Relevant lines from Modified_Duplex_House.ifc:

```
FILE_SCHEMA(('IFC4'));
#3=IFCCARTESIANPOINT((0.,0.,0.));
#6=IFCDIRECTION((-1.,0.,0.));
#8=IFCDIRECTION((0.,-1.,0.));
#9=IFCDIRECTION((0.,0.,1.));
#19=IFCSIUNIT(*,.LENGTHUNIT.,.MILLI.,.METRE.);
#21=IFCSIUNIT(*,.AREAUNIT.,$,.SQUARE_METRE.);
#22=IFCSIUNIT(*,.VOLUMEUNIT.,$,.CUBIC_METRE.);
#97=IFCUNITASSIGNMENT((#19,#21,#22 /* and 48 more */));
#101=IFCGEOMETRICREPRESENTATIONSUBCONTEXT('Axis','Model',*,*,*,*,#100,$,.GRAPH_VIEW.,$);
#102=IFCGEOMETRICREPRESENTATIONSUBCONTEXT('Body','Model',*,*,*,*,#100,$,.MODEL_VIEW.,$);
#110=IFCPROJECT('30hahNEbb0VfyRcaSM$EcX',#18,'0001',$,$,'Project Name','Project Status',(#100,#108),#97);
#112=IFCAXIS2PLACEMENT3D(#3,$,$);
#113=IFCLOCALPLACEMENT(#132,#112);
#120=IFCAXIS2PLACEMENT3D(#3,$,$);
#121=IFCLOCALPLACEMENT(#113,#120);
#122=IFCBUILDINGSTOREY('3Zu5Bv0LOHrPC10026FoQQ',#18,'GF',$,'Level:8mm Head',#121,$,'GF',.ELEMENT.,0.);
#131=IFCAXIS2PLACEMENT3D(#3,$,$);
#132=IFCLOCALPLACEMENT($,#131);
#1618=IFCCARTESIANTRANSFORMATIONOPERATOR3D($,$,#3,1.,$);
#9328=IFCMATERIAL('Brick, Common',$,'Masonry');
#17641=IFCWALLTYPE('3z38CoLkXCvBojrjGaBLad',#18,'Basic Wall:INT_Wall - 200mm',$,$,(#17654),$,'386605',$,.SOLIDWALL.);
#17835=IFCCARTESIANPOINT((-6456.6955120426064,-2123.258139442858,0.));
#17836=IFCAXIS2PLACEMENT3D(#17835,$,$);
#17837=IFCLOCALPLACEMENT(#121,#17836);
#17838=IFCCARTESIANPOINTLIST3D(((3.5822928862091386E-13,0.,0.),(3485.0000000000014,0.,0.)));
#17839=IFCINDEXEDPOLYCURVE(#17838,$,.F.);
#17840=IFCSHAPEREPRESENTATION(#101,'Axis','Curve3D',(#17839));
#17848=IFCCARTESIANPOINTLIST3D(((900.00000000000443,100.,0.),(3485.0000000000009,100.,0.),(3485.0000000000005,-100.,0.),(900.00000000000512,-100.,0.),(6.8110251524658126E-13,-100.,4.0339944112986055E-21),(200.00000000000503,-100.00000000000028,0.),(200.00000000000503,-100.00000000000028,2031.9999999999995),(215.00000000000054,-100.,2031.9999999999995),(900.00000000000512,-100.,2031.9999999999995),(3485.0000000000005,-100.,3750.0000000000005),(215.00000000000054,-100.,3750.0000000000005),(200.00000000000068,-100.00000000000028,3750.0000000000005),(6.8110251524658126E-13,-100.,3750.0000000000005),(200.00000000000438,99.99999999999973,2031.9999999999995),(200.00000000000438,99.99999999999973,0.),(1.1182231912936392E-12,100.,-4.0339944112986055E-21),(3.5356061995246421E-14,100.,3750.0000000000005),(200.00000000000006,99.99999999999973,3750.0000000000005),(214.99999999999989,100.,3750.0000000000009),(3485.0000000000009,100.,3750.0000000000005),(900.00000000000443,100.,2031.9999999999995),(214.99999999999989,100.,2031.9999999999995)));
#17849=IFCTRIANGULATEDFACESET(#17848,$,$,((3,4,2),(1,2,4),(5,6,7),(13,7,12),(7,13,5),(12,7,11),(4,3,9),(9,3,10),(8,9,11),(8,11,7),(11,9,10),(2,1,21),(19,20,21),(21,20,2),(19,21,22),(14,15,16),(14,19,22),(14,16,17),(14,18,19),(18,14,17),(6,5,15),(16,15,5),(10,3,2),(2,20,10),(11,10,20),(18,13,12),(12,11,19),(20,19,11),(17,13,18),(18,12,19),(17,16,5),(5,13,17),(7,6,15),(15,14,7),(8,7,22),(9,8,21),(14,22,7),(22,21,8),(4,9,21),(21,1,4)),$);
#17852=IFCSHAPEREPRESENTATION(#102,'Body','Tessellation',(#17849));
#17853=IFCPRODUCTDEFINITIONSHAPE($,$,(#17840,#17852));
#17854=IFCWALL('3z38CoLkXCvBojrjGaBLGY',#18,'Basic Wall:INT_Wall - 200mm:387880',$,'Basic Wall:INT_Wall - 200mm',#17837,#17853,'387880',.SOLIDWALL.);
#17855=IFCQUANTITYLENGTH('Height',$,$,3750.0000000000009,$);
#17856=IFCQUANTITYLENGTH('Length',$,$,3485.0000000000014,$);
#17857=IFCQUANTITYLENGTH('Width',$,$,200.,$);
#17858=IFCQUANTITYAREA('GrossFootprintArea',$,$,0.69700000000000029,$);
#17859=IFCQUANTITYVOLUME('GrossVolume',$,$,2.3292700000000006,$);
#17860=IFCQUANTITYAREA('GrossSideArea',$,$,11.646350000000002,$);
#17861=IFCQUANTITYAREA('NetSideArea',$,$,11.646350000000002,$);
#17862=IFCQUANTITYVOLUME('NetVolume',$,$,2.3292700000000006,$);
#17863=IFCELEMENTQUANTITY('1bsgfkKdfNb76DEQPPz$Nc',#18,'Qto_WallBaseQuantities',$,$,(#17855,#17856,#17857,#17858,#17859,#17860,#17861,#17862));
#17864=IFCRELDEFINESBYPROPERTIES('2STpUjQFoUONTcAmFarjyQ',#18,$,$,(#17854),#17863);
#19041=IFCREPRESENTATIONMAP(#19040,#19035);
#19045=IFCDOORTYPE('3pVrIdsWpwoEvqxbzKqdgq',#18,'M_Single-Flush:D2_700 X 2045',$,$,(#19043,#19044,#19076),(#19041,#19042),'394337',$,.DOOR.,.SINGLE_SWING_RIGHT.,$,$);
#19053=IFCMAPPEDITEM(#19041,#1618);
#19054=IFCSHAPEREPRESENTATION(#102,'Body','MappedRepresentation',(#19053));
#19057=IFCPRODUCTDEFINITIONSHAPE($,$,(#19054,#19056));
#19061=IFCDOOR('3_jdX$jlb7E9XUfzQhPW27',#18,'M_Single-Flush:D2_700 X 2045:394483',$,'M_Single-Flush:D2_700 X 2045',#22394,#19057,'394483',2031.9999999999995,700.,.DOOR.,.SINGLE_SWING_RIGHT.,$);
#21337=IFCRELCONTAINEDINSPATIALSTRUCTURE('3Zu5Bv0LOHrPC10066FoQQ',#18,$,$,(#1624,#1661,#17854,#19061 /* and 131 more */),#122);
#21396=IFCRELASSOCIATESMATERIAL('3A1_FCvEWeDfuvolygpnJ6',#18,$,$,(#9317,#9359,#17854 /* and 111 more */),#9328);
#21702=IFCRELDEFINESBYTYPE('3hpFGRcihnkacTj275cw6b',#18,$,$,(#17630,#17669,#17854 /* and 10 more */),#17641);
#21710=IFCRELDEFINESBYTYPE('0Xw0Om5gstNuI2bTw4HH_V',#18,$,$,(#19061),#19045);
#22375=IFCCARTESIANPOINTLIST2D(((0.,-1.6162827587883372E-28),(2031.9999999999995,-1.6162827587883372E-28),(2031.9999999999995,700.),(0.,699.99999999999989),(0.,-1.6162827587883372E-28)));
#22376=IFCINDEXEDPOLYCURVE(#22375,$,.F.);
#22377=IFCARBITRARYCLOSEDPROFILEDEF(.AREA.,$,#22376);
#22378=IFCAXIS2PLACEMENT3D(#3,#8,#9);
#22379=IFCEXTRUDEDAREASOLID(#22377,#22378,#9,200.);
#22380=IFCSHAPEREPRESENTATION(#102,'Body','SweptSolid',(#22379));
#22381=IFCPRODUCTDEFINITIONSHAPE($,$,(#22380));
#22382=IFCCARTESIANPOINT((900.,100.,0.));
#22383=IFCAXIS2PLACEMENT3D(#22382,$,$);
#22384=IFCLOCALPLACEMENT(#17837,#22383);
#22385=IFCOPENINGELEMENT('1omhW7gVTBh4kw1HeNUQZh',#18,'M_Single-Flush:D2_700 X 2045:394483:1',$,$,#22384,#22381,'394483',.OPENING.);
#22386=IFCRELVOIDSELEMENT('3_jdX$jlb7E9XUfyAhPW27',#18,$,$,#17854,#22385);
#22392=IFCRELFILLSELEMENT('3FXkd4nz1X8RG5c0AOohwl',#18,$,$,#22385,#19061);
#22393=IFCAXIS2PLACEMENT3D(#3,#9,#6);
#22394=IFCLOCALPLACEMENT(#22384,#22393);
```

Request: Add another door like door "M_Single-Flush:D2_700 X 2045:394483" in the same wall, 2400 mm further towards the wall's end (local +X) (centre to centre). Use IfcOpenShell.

```python
import ifcopenshell
import ifcopenshell.api.feature
import ifcopenshell.api.geometry
import ifcopenshell.api.pset
import ifcopenshell.api.root
import ifcopenshell.geom
import ifcopenshell.util.element
import ifcopenshell.util.placement
import ifcopenshell.util.shape
import ifcopenshell.util.unit

model = ifcopenshell.open("Modified_Duplex_House.ifc")
unit_scale = ifcopenshell.util.unit.calculate_unit_scale(model)
area_scale = ifcopenshell.util.unit.calculate_unit_scale(model, "AREAUNIT")
volume_scale = ifcopenshell.util.unit.calculate_unit_scale(model, "VOLUMEUNIT")
settings = ifcopenshell.geom.settings()


def volume(element):
    """Net volume in cubic metres, openings subtracted."""
    shape = ifcopenshell.geom.create_shape(settings, element)
    return ifcopenshell.util.shape.get_volume(shape.geometry)


def reuse_history(source, copy):
    """copy_class also copies each property set's owner history, people and application; keep the originals."""
    for rel in copy.IsDefinedBy:
        if rel.is_a("IfcRelDefinesByProperties") and (history := rel.RelatingPropertyDefinition.OwnerHistory):
            rel.RelatingPropertyDefinition.OwnerHistory = source.OwnerHistory
            ifcopenshell.util.element.remove_deep2(model, history)


door = model.by_guid("3_jdX$jlb7E9XUfzQhPW27")
opening = door.FillsVoids[0].RelatingOpeningElement
wall = opening.VoidsElements[0].RelatingBuildingElement
before = volume(wall)
shift = ifcopenshell.util.placement.get_local_placement(wall.ObjectPlacement)[:3, 0] * 2.4 / unit_scale

# copy_class copies the void relationship, type, container and properties, but no geometry.
new_opening = ifcopenshell.api.root.copy_class(model, product=opening)
new_opening.Representation = ifcopenshell.util.element.copy_deep(
    model, opening.Representation, exclude=["IfcGeometricRepresentationContext", "IfcRepresentationMap"]
)
new_opening.Name = "M_Single-Flush:D2_700 X 2045"
new_opening.Tag = None
reuse_history(opening, new_opening)
new_door = ifcopenshell.api.root.copy_class(model, product=door)
new_door.Representation = ifcopenshell.util.element.copy_deep(
    model, door.Representation, exclude=["IfcGeometricRepresentationContext", "IfcRepresentationMap"]
)
new_door.Name = "M_Single-Flush:D2_700 X 2045"
new_door.Tag = None
reuse_history(door, new_door)
ifcopenshell.api.feature.add_filling(model, opening=new_opening, element=new_door)

for old, new in ((opening, new_opening), (door, new_door)):
    matrix = ifcopenshell.util.placement.get_local_placement(old.ObjectPlacement)
    matrix[:3, 3] += shift
    ifcopenshell.api.geometry.edit_object_placement(model, product=new, matrix=matrix, is_si=False)

after = volume(wall)
thickness = 0.2  # wall thickness in metres

# Update the wall's stored quantities.
qto = model.by_id(ifcopenshell.util.element.get_pset(wall, "Qto_WallBaseQuantities", should_inherit=False)["id"])
ifcopenshell.api.pset.edit_qto(model, qto=qto, properties={
    "NetSideArea": after / thickness / area_scale,
    "NetVolume": after / volume_scale,
})

print(f"wall volume {before:.3f} -> {after:.3f} m3")

model.write("Modified_Duplex_House_edited.ifc")
```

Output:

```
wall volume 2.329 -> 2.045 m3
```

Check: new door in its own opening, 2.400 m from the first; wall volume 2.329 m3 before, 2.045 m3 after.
